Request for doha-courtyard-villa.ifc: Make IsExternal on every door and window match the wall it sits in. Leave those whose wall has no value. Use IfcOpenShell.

First a look at what the model holds.

```python
import ifcopenshell
import ifcopenshell.util.element

model = ifcopenshell.open("doha-courtyard-villa.ifc")
print(model.schema)
seen = {}
for e in model.by_type("IfcDoor") + model.by_type("IfcWindow"):
    if not e.FillsVoids:
        continue
    host = e.FillsVoids[0].RelatingOpeningElement.VoidsElements[0].RelatingBuildingElement
    own = ifcopenshell.util.element.get_pset(e, f"Pset_{e.is_a()[3:].removesuffix('StandardCase')}Common", "IsExternal")
    wall = ifcopenshell.util.element.get_pset(host, "Pset_WallCommon", "IsExternal")
    seen[e.is_a(), own, wall] = seen.get((e.is_a(), own, wall), 0) + 1
for (cls, own, wall), count in sorted(seen.items(), key=str):
    print(count, cls, "IsExternal:", own, "| host wall:", wall)
```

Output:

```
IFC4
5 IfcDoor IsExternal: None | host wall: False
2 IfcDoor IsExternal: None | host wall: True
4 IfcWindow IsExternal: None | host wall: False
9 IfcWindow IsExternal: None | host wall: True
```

```python
import ifcopenshell
import ifcopenshell.api.pset
import ifcopenshell.util.element

model = ifcopenshell.open("doha-courtyard-villa.ifc")

count = 0
for ifc_class, pset_name in (("IfcDoor", "Pset_DoorCommon"), ("IfcWindow", "Pset_WindowCommon")):
    for e in model.by_type(ifc_class):
        if not e.FillsVoids:
            continue
        host = e.FillsVoids[0].RelatingOpeningElement.VoidsElements[0].RelatingBuildingElement
        external = ifcopenshell.util.element.get_pset(host, "Pset_WallCommon", "IsExternal")
        if external is None or ifcopenshell.util.element.get_pset(e, pset_name, "IsExternal") == external:
            continue
        pset = ifcopenshell.api.pset.add_pset(model, product=e, name=pset_name)
        ifcopenshell.api.pset.edit_pset(model, pset=pset, properties={"IsExternal": external})
        count += 1

print(count, "updated")

model.write("doha-courtyard-villa_updated.ifc")
```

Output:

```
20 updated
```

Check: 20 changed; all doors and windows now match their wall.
